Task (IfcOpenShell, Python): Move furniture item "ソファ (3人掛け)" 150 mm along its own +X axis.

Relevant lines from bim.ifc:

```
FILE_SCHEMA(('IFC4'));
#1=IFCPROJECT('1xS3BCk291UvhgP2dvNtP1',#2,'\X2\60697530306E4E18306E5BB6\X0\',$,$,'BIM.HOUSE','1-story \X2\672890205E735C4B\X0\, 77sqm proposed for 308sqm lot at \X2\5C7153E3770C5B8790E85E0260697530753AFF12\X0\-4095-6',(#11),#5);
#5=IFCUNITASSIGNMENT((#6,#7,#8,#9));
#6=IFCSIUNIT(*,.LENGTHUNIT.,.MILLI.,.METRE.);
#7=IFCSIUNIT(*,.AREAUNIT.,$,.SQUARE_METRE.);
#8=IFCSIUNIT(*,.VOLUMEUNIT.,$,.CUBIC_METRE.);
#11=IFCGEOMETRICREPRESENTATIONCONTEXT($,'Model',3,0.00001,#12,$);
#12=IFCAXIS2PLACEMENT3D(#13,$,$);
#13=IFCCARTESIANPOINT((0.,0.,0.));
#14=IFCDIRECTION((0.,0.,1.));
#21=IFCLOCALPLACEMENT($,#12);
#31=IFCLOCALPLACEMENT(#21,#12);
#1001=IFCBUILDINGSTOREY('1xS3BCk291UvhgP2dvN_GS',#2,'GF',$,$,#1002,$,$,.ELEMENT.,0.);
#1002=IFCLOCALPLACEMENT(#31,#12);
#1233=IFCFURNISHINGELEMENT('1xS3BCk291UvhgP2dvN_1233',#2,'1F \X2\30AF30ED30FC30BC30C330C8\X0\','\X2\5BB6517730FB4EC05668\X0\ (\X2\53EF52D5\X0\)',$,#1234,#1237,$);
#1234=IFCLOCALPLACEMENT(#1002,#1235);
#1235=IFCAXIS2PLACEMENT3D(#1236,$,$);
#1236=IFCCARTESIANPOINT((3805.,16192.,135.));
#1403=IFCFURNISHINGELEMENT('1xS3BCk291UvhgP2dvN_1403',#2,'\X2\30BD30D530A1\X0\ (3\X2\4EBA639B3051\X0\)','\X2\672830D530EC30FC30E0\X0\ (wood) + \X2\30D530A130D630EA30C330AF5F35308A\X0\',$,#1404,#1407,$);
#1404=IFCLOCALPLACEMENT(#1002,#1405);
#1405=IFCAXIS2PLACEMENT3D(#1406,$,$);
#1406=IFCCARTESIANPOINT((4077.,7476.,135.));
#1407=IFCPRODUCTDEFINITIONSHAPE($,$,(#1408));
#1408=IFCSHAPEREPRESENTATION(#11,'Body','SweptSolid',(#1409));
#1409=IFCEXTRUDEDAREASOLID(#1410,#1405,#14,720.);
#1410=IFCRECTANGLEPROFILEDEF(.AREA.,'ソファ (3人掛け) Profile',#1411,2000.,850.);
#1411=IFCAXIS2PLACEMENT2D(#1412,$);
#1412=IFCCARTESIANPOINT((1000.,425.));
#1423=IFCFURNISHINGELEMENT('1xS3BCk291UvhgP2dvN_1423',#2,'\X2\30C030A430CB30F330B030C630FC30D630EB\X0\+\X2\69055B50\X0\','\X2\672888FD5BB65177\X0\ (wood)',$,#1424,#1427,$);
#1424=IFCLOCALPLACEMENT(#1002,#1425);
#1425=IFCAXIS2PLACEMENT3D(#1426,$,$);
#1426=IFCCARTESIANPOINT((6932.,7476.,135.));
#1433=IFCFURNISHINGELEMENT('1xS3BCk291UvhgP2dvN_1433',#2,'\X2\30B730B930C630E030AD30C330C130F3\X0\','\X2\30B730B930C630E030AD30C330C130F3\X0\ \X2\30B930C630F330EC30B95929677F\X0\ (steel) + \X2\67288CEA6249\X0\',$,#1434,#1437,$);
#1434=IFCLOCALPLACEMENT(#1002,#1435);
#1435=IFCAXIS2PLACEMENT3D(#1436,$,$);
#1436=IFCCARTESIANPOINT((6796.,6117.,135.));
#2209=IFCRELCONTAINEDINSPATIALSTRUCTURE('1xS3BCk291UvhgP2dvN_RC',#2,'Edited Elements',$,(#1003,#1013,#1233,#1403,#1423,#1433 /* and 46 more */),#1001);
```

```python
import ifcopenshell
import ifcopenshell.api.geometry
import ifcopenshell.util.placement

model = ifcopenshell.open("bim.ifc")

item = model.by_id(1403)
matrix = ifcopenshell.util.placement.get_local_placement(item.ObjectPlacement)
matrix[:3, 3] += matrix[:3, 0] * 150.0
ifcopenshell.api.geometry.edit_object_placement(model, product=item, matrix=matrix, is_si=False)

print(ifcopenshell.util.placement.get_local_placement(item.ObjectPlacement).round(3) + 0.0)

model.write("bim-out.ifc")
```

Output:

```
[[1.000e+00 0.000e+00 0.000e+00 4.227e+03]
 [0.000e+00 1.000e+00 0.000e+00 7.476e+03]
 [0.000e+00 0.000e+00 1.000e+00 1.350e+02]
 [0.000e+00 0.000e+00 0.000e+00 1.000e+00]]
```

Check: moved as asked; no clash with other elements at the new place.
